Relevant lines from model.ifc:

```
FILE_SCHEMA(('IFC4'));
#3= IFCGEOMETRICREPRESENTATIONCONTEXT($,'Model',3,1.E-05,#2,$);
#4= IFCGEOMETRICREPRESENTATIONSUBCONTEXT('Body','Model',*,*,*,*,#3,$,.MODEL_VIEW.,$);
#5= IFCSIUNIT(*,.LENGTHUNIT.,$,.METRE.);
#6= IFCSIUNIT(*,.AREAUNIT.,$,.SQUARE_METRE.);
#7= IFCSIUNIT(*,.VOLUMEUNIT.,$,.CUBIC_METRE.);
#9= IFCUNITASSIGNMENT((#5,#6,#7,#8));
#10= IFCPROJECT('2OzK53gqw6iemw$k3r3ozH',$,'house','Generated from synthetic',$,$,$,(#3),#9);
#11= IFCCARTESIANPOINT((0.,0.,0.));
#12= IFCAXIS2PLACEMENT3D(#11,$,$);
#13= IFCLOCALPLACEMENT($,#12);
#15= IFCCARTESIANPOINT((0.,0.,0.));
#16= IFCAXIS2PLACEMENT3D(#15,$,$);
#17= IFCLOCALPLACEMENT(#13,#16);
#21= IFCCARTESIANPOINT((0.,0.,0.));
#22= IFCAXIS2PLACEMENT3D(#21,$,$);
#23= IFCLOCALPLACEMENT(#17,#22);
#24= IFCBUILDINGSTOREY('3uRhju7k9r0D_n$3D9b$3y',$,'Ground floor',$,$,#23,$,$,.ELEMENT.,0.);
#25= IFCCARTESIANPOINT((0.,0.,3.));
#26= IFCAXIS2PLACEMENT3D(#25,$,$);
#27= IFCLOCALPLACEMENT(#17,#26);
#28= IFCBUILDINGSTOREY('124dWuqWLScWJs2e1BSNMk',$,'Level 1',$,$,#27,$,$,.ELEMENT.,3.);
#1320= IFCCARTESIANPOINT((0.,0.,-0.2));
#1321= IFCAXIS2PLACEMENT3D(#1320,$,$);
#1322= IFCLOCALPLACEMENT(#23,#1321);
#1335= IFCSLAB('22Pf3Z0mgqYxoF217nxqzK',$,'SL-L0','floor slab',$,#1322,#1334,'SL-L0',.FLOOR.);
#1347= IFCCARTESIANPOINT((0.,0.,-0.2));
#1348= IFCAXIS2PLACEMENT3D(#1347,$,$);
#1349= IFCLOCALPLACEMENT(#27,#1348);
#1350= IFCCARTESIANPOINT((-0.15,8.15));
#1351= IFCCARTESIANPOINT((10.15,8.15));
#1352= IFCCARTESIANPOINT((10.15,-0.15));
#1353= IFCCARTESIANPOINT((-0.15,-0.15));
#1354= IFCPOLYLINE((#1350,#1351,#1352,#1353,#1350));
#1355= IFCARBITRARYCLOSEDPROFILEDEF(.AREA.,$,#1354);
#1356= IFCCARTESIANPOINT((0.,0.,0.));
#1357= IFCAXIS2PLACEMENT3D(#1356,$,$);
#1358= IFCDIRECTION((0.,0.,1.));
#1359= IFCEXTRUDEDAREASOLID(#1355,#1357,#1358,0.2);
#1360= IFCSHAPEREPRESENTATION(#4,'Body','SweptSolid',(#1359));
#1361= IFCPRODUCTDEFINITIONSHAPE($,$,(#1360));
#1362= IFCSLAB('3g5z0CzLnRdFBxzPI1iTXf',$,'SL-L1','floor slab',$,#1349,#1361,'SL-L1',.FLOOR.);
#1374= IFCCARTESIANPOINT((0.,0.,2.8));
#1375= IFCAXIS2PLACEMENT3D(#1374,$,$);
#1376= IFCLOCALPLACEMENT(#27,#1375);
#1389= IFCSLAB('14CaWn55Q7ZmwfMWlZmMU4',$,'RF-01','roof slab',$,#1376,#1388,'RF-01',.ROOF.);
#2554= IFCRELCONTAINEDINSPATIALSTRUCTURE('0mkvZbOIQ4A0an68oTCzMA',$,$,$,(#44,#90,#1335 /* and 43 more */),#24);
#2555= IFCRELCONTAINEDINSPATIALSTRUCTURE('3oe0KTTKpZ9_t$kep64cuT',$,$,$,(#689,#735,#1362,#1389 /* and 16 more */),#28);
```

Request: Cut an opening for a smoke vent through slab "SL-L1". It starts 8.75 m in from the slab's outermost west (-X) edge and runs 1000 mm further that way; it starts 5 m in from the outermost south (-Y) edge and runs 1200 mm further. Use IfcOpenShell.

```python
import numpy as np
import ifcopenshell
import ifcopenshell.api.feature
import ifcopenshell.api.geometry
import ifcopenshell.api.root
import ifcopenshell.geom
import ifcopenshell.util.placement
import ifcopenshell.util.representation
import ifcopenshell.util.shape
import ifcopenshell.util.unit

model = ifcopenshell.open("model.ifc")
unit_scale = ifcopenshell.util.unit.calculate_unit_scale(model)
settings = ifcopenshell.geom.settings()


def volume(element):
    """Net volume in cubic metres, openings subtracted."""
    shape = ifcopenshell.geom.create_shape(settings, element)
    return ifcopenshell.util.shape.get_volume(shape.geometry)


slab = model.by_guid("3g5z0CzLnRdFBxzPI1iTXf")
before = volume(slab)

# Extent in the slab's own axes, in metres. The edges named are its -X and -Y sides.
slab_shape = ifcopenshell.geom.create_shape(settings, slab)
vertices = ifcopenshell.util.shape.get_vertices(slab_shape.geometry)
x_min, y_min, bottom = vertices.min(axis=0)
top = vertices[:, 2].max()

opening = ifcopenshell.api.root.create_entity(model, ifc_class="IfcOpeningElement", name="Smoke vent opening", predefined_type="OPENING")
context = ifcopenshell.util.representation.get_context(model, "Model", "Body", "MODEL_VIEW")
width, depth = 1, 1.2
outline = [(0.0, 0.0), (width, 0.0), (width, depth), (0.0, depth), (0.0, 0.0)]
# Overshoot both faces by 50 mm so the cut is clean.
shape = ifcopenshell.api.geometry.add_slab_representation(
    model, context=context, depth=top - bottom + 0.1, polyline=outline
)
ifcopenshell.api.geometry.assign_representation(model, product=opening, representation=shape)

matrix = ifcopenshell.util.placement.get_local_placement(slab.ObjectPlacement)
matrix[:, 3] = matrix @ np.append(np.array([x_min + 8.75, y_min + 5, bottom - 0.05]) / unit_scale, 1.0)
ifcopenshell.api.geometry.edit_object_placement(model, product=opening, matrix=matrix, is_si=False)
ifcopenshell.api.feature.add_feature(model, feature=opening, element=slab)

after = volume(slab)

print(f"slab volume {before:.3f} -> {after:.3f} m3")

model.write("model_rev.ifc")
```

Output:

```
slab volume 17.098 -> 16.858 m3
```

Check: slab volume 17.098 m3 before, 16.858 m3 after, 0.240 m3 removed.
